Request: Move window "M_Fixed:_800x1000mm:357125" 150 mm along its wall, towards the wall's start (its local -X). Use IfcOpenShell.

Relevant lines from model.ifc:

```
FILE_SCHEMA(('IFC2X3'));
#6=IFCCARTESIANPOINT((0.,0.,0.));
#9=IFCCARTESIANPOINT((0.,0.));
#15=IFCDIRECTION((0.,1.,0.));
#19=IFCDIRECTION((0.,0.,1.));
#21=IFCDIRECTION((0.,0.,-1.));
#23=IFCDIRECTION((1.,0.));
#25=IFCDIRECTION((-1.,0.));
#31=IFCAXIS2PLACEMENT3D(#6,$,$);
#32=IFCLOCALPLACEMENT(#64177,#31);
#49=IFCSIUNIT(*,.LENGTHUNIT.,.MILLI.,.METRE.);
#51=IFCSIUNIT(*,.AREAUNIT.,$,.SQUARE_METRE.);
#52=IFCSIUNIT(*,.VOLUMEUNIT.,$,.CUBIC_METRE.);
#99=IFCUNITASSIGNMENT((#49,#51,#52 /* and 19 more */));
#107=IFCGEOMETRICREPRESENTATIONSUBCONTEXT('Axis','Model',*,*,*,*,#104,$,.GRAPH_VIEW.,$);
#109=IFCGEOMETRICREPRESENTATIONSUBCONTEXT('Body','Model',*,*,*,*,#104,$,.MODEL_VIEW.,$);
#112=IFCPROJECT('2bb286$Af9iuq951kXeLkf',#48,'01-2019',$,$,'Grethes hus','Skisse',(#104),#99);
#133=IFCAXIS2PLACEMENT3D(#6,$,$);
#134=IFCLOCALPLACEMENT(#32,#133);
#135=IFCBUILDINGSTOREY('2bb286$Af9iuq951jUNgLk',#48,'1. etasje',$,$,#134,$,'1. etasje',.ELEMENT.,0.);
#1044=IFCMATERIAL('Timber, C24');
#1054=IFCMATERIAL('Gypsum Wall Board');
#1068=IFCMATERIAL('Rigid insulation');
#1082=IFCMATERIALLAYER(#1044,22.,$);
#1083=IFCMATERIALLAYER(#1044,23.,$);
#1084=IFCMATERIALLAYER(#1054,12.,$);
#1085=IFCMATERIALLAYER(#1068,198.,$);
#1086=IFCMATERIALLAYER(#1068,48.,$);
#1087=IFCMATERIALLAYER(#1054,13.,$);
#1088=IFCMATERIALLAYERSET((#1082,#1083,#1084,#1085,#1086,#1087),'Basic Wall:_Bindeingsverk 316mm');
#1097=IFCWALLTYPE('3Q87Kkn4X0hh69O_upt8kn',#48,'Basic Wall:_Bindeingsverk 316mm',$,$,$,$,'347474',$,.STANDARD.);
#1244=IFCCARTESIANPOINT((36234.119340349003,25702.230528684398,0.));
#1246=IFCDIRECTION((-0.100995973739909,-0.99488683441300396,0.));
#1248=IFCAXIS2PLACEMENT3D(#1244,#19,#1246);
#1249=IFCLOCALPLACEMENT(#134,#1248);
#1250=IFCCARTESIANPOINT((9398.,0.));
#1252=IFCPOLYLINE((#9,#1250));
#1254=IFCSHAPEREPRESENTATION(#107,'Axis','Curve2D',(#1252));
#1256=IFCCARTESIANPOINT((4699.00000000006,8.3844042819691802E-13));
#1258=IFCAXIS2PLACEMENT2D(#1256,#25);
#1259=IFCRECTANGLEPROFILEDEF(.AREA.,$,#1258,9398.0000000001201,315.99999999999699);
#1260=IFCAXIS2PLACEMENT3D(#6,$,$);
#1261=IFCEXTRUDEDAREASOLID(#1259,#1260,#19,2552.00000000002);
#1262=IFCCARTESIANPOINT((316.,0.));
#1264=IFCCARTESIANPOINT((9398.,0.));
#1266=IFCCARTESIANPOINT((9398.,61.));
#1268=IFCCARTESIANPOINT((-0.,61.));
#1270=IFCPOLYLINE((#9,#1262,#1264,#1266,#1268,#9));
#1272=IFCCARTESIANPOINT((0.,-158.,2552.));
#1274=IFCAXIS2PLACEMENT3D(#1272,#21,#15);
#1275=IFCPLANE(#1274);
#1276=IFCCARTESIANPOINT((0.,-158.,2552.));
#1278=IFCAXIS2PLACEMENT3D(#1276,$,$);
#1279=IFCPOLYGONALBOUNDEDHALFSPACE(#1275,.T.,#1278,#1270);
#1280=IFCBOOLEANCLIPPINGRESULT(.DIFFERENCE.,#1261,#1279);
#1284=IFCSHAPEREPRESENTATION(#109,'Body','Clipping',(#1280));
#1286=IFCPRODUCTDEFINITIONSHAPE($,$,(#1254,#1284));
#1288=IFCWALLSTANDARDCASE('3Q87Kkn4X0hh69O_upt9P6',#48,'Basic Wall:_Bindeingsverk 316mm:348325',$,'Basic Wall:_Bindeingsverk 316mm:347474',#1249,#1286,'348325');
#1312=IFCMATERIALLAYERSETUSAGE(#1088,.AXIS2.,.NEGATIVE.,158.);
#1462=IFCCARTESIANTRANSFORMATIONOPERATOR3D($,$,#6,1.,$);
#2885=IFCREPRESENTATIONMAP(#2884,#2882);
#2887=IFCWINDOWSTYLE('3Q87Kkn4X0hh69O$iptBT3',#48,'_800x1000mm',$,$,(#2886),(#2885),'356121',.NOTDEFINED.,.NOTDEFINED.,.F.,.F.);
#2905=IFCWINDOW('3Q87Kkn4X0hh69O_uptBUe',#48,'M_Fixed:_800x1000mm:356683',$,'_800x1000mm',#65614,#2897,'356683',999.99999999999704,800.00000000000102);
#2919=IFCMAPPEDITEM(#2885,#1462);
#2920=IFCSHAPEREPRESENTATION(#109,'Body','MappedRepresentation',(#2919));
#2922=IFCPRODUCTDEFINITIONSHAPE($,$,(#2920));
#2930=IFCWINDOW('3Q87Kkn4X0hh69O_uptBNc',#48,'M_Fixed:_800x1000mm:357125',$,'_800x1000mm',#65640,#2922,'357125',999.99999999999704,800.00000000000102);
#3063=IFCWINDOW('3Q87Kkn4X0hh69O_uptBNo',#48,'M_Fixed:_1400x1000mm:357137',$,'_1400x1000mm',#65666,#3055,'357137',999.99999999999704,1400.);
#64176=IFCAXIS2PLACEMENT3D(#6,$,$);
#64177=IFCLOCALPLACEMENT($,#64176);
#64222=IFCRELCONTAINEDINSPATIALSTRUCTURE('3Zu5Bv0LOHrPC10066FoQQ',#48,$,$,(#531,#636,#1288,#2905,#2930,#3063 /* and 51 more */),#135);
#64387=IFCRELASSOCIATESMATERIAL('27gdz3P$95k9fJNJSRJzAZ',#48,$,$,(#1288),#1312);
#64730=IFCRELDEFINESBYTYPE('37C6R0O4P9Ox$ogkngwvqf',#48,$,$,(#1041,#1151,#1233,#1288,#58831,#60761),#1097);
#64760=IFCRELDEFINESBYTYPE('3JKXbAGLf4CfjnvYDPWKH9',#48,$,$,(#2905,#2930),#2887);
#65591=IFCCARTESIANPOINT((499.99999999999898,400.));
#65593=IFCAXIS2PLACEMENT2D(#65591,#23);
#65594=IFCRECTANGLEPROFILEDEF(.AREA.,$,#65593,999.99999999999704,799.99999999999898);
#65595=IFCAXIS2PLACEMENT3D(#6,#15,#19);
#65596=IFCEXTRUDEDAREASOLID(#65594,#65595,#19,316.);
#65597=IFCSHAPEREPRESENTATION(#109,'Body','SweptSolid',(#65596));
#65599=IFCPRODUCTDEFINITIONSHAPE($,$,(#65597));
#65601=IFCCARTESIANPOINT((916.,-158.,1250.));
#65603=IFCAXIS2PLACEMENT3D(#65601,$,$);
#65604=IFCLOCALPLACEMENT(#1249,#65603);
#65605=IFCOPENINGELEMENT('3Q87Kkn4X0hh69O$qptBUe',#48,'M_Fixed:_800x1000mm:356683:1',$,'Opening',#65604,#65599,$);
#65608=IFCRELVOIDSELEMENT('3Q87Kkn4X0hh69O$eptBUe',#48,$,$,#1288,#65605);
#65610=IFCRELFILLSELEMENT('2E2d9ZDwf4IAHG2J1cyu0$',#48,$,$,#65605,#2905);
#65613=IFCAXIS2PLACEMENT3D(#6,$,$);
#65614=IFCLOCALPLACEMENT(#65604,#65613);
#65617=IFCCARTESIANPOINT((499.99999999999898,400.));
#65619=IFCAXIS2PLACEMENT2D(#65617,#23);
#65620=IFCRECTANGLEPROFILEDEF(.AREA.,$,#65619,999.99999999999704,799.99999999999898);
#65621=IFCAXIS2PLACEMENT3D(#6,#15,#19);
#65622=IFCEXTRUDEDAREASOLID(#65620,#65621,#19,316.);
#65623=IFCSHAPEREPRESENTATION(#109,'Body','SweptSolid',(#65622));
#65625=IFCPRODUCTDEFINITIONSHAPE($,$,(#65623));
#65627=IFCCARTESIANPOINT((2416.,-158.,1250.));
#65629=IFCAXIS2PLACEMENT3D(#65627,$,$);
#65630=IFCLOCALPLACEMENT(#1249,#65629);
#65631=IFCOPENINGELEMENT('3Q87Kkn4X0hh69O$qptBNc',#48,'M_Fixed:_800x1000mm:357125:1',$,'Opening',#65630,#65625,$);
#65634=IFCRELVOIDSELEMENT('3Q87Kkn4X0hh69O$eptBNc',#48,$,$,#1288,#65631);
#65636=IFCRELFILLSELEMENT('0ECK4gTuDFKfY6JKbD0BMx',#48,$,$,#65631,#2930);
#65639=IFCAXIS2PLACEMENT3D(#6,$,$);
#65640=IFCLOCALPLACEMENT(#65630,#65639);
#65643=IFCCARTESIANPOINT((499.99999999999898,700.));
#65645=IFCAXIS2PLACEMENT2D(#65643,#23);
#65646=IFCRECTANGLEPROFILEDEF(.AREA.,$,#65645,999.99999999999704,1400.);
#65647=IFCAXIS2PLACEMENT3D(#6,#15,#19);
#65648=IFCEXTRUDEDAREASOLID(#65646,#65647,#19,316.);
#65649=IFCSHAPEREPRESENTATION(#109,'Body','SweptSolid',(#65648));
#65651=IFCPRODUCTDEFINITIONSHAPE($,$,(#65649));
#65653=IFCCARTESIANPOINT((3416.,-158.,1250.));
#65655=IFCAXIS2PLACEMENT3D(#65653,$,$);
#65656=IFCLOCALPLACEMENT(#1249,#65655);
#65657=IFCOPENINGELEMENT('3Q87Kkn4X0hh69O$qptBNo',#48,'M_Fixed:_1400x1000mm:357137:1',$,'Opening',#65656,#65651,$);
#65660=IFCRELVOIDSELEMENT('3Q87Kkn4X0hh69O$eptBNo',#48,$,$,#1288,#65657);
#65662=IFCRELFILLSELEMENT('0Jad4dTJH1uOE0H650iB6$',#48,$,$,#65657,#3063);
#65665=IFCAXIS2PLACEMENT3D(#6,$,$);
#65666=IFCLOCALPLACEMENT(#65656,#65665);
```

```python
import ifcopenshell
import ifcopenshell.api.geometry
import ifcopenshell.util.placement
import ifcopenshell.util.unit

model = ifcopenshell.open("model.ifc")
unit_scale = ifcopenshell.util.unit.calculate_unit_scale(model)

window = model.by_guid("3Q87Kkn4X0hh69O_uptBNc")
opening = window.FillsVoids[0].RelatingOpeningElement
wall = opening.VoidsElements[0].RelatingBuildingElement

wall_matrix = ifcopenshell.util.placement.get_local_placement(wall.ObjectPlacement)
shift = wall_matrix[:3, 0] * -0.15 / unit_scale
before = ifcopenshell.util.placement.get_local_placement(window.ObjectPlacement)[:3, 3].copy()

# The window is placed relative to its opening, so it follows when the opening moves.
matrix = ifcopenshell.util.placement.get_local_placement(opening.ObjectPlacement)
matrix[:3, 3] += shift
ifcopenshell.api.geometry.edit_object_placement(
    model, product=opening, matrix=matrix, is_si=False, should_transform_children=True
)

after = ifcopenshell.util.placement.get_local_placement(window.ObjectPlacement)[:3, 3]
print("window moved by", (after - before).round(3) + 0.0)

model.write("model_updated.ifc")
```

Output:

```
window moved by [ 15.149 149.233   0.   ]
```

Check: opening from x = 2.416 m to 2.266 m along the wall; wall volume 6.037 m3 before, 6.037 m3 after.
